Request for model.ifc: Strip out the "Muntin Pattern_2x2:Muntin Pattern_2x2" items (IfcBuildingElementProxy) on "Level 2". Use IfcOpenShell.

First a look at what the model holds.

```python
import ifcopenshell
import ifcopenshell.util.element

model = ifcopenshell.open("model.ifc")
print(model.schema)
storey = next(s for s in model.by_type("IfcBuildingStorey") if s.Name == "Level 2")
proxies = [e for e in ifcopenshell.util.element.get_decomposition(storey) if e.is_a("IfcBuildingElementProxy")]
seen = {}
for e in proxies:
    element_type = ifcopenshell.util.element.get_type(e)
    name = element_type.Name if element_type not in (None, e) else None
    seen[name] = seen.get(name, 0) + 1
for name, count in sorted(seen.items(), key=str):
    print(count, "x", name)
```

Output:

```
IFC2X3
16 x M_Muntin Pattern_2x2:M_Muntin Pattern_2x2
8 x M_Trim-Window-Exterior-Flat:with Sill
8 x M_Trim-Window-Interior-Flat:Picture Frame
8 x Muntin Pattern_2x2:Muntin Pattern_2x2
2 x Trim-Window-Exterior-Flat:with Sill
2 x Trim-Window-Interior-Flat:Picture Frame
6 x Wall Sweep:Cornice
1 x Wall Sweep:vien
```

```python
import ifcopenshell
import ifcopenshell.api.root
import ifcopenshell.util.element

model = ifcopenshell.open("model.ifc")

storey = next(s for s in model.by_type("IfcBuildingStorey") if s.Name == "Level 2")
proxies = [e for e in ifcopenshell.util.element.get_decomposition(storey) if e.is_a("IfcBuildingElementProxy")]
targets = [e for e in proxies if (t := ifcopenshell.util.element.get_type(e)) not in (None, e) and t.Name == "Muntin Pattern_2x2:Muntin Pattern_2x2"]

for e in targets:
    ifcopenshell.api.root.remove_product(model, product=e)
print(len(targets), "removed")

model.write("model_updated.ifc")
```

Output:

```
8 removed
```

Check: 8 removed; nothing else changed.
